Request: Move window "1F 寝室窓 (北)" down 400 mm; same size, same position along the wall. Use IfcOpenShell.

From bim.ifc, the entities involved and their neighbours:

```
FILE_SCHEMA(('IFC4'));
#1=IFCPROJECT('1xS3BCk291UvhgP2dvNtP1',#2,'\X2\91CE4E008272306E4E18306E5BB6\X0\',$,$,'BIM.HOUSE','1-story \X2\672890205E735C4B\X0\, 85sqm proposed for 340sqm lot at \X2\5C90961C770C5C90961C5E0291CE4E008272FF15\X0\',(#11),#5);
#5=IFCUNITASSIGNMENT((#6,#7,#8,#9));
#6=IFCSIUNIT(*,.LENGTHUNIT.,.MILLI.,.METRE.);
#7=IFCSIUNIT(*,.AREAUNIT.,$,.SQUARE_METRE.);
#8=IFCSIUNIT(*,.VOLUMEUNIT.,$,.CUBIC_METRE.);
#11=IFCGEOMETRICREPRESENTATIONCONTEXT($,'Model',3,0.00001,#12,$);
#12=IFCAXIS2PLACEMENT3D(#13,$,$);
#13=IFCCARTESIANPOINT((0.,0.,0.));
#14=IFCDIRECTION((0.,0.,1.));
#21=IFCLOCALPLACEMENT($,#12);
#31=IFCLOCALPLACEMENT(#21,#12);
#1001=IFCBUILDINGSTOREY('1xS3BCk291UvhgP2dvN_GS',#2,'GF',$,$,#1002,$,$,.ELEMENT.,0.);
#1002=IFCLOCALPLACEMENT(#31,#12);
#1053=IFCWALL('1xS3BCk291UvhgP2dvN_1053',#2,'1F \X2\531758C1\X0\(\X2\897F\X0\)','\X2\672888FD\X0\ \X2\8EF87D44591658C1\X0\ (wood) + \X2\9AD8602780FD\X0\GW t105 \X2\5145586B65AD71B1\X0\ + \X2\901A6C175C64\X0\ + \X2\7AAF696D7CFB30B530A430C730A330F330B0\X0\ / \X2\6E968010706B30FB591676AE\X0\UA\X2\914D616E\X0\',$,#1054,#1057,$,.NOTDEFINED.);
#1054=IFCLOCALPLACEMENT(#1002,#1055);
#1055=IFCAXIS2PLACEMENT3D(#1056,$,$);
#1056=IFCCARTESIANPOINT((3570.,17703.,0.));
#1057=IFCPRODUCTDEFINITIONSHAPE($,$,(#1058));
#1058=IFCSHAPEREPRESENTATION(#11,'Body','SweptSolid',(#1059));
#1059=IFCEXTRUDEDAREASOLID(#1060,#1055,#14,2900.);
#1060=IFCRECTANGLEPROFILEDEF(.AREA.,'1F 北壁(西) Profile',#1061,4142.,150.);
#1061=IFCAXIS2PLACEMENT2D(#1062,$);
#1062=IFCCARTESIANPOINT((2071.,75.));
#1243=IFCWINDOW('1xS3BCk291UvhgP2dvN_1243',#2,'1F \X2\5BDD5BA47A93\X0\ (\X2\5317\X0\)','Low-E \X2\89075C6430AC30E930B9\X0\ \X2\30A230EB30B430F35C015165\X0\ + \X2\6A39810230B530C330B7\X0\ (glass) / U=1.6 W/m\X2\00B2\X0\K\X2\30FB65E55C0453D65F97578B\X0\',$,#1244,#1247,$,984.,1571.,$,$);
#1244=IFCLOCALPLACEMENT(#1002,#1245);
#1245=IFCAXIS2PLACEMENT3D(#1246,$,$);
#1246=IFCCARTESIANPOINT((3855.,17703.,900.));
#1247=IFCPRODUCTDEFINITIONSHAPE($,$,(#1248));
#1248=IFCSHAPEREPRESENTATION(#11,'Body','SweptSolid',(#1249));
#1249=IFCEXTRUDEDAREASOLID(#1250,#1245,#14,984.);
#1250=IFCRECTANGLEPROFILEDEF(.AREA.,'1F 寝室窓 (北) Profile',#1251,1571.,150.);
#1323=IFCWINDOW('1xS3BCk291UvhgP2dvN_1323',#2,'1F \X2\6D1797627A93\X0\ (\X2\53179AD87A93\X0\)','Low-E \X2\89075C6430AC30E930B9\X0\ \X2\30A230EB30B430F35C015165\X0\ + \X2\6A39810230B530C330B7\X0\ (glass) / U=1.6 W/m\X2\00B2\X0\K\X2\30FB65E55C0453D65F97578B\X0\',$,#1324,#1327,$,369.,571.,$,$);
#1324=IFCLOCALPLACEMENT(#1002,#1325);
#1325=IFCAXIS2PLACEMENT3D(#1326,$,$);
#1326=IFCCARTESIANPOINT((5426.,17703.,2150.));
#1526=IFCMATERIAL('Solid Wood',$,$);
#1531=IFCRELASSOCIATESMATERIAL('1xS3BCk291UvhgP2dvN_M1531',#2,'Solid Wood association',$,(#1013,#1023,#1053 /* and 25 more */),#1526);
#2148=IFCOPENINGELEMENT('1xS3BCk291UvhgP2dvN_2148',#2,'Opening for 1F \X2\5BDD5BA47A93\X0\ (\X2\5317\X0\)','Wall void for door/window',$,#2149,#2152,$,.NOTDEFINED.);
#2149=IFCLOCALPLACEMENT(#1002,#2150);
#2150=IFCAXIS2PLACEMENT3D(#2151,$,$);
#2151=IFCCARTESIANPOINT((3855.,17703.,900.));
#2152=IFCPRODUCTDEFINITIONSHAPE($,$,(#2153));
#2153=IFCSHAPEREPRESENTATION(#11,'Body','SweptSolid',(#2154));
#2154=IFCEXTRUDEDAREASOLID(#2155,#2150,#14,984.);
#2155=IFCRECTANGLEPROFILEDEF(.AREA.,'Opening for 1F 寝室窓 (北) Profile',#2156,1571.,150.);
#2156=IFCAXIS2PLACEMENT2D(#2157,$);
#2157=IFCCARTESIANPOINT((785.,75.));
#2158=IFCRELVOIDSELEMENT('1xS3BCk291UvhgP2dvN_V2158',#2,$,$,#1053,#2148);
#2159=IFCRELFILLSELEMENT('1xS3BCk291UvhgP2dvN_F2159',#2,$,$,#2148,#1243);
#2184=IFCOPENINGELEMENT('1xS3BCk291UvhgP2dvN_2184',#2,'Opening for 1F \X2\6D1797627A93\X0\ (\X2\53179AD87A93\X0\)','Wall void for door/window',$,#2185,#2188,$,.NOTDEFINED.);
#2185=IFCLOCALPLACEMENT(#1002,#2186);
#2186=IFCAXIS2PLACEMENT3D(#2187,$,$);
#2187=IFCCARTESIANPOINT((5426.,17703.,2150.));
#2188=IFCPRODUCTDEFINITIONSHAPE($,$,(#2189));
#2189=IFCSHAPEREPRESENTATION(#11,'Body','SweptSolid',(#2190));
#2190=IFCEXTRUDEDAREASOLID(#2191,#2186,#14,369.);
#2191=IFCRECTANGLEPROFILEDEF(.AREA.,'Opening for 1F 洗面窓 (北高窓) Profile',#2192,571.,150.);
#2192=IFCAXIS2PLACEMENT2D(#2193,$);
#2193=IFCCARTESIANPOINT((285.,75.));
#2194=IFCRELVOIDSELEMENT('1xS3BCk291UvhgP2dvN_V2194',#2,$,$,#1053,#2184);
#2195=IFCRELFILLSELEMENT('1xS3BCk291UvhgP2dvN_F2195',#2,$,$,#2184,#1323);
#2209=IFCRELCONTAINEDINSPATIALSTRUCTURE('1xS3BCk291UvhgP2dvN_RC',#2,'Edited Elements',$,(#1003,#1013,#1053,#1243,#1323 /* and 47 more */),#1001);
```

```python
import numpy as np
import ifcopenshell
import ifcopenshell.api.geometry
import ifcopenshell.util.placement
import ifcopenshell.util.unit

model = ifcopenshell.open("bim.ifc")
unit_scale = ifcopenshell.util.unit.calculate_unit_scale(model)

window = model.by_guid("1xS3BCk291UvhgP2dvN_1243")
opening = window.FillsVoids[0].RelatingOpeningElement
dz = -400.0

shift = np.array([0.0, 0.0, dz])
# The window is not placed relative to its opening, so move both.
for product in (opening, window):
    matrix = ifcopenshell.util.placement.get_local_placement(product.ObjectPlacement)
    matrix[:3, 3] += shift
    ifcopenshell.api.geometry.edit_object_placement(model, product=product, matrix=matrix, is_si=False)

print(f"moved by {dz * unit_scale:+.3f} m")

model.write("bim_edited.ifc")
```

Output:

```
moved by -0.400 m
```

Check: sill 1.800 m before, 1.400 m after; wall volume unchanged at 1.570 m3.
